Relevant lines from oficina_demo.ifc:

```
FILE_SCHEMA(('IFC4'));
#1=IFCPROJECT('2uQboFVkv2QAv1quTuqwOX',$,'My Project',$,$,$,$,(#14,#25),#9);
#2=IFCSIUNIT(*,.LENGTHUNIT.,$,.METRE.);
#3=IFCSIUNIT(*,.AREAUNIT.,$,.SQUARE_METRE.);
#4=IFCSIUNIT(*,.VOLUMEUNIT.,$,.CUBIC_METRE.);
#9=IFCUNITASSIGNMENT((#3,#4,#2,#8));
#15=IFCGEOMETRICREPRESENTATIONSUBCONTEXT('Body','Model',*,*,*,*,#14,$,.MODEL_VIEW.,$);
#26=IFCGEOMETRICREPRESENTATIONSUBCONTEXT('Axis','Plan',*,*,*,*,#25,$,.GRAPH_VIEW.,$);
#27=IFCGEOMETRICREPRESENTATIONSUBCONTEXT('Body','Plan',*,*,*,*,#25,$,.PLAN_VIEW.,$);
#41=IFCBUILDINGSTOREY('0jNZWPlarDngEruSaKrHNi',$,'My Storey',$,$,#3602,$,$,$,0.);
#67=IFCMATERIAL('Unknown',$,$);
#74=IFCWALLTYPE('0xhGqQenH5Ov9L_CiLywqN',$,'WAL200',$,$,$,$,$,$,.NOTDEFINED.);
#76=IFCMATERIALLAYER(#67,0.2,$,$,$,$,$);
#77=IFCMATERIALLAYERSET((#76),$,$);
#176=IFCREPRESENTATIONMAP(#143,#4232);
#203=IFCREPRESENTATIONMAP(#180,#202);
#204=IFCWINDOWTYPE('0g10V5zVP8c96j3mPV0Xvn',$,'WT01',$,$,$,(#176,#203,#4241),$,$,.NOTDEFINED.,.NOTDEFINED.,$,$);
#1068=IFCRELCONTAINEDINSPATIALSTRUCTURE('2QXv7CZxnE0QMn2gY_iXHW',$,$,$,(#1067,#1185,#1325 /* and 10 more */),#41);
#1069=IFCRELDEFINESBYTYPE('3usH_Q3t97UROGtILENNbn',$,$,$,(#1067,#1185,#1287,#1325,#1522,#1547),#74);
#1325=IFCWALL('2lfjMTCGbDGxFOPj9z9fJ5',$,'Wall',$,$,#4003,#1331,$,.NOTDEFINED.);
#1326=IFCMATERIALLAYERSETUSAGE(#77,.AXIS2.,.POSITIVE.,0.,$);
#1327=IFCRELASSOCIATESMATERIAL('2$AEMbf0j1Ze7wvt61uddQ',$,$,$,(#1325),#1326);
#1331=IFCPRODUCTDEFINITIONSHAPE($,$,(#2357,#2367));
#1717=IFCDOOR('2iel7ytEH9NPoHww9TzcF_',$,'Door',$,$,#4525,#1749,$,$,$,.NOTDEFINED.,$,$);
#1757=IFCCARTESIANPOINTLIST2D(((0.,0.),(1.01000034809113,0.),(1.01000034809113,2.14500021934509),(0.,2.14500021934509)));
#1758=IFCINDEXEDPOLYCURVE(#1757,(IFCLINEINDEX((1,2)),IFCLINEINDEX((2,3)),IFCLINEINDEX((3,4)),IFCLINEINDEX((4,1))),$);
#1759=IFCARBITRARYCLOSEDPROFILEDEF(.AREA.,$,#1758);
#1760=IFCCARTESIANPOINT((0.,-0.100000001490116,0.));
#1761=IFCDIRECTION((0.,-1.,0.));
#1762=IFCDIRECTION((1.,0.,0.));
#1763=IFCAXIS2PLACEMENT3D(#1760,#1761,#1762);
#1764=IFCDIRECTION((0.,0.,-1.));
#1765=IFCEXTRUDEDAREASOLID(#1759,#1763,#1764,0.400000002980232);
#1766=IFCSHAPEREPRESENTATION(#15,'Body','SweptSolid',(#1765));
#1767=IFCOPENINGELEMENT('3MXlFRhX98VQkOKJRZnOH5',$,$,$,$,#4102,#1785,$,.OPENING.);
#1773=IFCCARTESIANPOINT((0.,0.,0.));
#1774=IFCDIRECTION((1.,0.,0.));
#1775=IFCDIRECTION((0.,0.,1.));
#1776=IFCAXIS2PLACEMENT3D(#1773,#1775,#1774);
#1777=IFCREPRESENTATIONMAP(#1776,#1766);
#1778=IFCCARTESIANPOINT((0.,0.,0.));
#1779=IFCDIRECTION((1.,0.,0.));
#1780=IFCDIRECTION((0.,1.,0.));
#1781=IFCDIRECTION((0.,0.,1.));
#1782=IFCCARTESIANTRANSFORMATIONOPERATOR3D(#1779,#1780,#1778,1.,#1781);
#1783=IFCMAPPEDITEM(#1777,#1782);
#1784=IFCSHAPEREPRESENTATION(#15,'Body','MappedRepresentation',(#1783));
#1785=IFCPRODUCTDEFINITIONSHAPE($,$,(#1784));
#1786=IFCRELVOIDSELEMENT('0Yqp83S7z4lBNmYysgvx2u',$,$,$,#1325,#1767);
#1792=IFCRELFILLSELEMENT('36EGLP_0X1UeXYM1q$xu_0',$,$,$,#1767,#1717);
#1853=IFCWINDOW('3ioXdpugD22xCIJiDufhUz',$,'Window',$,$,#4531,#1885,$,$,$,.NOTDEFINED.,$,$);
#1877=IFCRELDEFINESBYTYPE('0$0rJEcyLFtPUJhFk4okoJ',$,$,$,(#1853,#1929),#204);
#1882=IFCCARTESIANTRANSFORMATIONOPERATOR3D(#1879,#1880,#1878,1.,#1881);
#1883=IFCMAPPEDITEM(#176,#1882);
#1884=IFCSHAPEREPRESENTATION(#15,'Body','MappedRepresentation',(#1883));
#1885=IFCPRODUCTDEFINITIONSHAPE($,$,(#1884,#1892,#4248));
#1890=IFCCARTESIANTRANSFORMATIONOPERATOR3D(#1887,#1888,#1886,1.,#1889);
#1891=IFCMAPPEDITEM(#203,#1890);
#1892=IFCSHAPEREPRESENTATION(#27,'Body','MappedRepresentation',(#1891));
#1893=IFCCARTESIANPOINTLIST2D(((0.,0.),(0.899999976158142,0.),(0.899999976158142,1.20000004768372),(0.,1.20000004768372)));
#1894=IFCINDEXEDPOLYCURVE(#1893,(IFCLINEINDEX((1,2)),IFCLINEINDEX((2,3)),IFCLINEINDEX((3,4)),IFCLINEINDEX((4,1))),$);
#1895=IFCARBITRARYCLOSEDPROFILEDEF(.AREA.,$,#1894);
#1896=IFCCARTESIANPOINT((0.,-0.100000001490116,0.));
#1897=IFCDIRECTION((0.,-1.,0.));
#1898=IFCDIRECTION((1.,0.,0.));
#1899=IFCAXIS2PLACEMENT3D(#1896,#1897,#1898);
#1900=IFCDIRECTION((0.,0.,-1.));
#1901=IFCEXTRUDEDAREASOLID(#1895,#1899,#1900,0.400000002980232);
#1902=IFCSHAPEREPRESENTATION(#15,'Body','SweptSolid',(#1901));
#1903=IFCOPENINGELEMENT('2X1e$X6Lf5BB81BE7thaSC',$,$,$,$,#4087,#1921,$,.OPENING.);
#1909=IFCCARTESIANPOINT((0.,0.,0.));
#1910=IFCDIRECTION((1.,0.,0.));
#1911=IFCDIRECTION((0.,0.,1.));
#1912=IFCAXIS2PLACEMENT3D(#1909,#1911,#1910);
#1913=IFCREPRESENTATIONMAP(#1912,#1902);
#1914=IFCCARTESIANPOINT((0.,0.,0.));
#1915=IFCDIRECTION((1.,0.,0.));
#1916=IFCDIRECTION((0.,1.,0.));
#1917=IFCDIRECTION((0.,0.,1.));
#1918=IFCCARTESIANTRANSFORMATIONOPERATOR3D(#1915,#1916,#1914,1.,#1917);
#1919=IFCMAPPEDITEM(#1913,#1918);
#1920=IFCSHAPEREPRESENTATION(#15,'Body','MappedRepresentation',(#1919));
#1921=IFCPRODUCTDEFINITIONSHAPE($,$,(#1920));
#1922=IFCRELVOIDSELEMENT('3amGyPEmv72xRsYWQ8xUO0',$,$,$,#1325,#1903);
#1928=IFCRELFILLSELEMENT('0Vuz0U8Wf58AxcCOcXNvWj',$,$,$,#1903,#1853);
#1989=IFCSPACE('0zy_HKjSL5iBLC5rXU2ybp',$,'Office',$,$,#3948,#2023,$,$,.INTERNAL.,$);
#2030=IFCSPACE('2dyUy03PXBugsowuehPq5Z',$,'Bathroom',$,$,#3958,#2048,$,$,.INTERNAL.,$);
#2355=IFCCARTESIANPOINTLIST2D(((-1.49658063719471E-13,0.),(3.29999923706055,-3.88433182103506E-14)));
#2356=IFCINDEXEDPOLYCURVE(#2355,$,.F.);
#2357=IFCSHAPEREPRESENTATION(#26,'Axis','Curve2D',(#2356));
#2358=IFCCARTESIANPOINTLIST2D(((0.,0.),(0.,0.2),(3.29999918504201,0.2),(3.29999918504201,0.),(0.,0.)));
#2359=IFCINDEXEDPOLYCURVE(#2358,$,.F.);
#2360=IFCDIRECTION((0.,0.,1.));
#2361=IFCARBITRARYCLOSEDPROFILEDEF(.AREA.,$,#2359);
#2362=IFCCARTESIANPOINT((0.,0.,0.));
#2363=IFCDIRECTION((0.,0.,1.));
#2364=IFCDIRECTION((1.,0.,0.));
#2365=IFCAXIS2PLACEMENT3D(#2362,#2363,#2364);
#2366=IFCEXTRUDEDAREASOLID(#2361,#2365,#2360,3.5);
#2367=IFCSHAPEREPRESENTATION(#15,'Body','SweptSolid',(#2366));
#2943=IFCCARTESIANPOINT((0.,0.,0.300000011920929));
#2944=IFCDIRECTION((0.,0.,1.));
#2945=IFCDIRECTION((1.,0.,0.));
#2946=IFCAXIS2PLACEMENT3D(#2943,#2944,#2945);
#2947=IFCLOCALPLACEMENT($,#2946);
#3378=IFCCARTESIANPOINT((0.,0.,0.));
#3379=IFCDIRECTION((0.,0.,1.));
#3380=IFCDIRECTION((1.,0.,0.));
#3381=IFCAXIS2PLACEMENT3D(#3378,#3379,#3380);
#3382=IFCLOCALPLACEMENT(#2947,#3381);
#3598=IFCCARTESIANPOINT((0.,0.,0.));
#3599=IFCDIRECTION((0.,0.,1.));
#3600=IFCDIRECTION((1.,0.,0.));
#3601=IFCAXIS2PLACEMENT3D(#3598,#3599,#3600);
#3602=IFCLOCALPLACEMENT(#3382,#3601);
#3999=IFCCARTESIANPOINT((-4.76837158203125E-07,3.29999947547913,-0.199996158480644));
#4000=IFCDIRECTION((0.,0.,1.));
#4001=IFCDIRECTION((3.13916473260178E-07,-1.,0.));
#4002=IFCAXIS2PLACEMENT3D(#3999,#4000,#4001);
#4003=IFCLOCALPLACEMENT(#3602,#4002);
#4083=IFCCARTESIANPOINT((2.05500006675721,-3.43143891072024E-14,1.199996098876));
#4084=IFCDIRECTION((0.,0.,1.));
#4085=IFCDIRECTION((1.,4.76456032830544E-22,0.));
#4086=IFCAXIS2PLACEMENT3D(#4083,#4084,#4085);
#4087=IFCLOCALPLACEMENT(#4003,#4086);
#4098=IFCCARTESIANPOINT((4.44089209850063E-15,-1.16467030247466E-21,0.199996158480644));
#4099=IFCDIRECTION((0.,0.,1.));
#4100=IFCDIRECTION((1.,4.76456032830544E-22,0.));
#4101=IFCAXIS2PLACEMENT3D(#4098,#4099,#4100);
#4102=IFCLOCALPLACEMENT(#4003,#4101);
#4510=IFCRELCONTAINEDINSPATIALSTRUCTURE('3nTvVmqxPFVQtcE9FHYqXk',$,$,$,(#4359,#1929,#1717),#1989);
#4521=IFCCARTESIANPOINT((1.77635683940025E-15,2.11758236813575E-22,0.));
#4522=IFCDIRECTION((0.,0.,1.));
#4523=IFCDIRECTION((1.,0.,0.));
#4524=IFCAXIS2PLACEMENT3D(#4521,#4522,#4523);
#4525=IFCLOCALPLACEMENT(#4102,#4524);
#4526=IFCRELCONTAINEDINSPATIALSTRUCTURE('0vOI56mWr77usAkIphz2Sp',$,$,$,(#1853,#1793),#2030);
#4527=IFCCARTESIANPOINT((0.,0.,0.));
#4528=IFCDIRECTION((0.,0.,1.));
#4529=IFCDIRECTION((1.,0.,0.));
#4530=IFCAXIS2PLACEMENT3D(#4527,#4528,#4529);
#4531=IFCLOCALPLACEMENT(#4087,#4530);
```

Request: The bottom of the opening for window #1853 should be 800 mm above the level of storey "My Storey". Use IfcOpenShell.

```python
import numpy as np
import ifcopenshell
import ifcopenshell.api.geometry
import ifcopenshell.geom
import ifcopenshell.util.element
import ifcopenshell.util.placement
import ifcopenshell.util.shape
import ifcopenshell.util.unit

model = ifcopenshell.open("oficina_demo.ifc")
unit_scale = ifcopenshell.util.unit.calculate_unit_scale(model)

window = model.by_guid("3ioXdpugD22xCIJiDufhUz")
opening = window.FillsVoids[0].RelatingOpeningElement
storey = ifcopenshell.util.element.get_container(window, ifc_class="IfcBuildingStorey")
level = ifcopenshell.util.placement.get_local_placement(storey.ObjectPlacement)[2, 3]

# The opening's origin need not be at the sill, so measure its lowest point.
shape = ifcopenshell.geom.create_shape(ifcopenshell.geom.settings(), opening)
bottom = ifcopenshell.util.shape.get_shape_bottom_elevation(shape, shape.geometry) / unit_scale
dz = level + 0.8 - bottom

shift = np.array([0.0, 0.0, dz])
# The window is placed relative to its opening, so it follows when the opening moves.
matrix = ifcopenshell.util.placement.get_local_placement(opening.ObjectPlacement)
matrix[:3, 3] += shift
ifcopenshell.api.geometry.edit_object_placement(
    model, product=opening, matrix=matrix, is_si=False, should_transform_children=True
)

print(f"moved by {dz * unit_scale:+.3f} m")

model.write("oficina_demo_edited.ifc")
```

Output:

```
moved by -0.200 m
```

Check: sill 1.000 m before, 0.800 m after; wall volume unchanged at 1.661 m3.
